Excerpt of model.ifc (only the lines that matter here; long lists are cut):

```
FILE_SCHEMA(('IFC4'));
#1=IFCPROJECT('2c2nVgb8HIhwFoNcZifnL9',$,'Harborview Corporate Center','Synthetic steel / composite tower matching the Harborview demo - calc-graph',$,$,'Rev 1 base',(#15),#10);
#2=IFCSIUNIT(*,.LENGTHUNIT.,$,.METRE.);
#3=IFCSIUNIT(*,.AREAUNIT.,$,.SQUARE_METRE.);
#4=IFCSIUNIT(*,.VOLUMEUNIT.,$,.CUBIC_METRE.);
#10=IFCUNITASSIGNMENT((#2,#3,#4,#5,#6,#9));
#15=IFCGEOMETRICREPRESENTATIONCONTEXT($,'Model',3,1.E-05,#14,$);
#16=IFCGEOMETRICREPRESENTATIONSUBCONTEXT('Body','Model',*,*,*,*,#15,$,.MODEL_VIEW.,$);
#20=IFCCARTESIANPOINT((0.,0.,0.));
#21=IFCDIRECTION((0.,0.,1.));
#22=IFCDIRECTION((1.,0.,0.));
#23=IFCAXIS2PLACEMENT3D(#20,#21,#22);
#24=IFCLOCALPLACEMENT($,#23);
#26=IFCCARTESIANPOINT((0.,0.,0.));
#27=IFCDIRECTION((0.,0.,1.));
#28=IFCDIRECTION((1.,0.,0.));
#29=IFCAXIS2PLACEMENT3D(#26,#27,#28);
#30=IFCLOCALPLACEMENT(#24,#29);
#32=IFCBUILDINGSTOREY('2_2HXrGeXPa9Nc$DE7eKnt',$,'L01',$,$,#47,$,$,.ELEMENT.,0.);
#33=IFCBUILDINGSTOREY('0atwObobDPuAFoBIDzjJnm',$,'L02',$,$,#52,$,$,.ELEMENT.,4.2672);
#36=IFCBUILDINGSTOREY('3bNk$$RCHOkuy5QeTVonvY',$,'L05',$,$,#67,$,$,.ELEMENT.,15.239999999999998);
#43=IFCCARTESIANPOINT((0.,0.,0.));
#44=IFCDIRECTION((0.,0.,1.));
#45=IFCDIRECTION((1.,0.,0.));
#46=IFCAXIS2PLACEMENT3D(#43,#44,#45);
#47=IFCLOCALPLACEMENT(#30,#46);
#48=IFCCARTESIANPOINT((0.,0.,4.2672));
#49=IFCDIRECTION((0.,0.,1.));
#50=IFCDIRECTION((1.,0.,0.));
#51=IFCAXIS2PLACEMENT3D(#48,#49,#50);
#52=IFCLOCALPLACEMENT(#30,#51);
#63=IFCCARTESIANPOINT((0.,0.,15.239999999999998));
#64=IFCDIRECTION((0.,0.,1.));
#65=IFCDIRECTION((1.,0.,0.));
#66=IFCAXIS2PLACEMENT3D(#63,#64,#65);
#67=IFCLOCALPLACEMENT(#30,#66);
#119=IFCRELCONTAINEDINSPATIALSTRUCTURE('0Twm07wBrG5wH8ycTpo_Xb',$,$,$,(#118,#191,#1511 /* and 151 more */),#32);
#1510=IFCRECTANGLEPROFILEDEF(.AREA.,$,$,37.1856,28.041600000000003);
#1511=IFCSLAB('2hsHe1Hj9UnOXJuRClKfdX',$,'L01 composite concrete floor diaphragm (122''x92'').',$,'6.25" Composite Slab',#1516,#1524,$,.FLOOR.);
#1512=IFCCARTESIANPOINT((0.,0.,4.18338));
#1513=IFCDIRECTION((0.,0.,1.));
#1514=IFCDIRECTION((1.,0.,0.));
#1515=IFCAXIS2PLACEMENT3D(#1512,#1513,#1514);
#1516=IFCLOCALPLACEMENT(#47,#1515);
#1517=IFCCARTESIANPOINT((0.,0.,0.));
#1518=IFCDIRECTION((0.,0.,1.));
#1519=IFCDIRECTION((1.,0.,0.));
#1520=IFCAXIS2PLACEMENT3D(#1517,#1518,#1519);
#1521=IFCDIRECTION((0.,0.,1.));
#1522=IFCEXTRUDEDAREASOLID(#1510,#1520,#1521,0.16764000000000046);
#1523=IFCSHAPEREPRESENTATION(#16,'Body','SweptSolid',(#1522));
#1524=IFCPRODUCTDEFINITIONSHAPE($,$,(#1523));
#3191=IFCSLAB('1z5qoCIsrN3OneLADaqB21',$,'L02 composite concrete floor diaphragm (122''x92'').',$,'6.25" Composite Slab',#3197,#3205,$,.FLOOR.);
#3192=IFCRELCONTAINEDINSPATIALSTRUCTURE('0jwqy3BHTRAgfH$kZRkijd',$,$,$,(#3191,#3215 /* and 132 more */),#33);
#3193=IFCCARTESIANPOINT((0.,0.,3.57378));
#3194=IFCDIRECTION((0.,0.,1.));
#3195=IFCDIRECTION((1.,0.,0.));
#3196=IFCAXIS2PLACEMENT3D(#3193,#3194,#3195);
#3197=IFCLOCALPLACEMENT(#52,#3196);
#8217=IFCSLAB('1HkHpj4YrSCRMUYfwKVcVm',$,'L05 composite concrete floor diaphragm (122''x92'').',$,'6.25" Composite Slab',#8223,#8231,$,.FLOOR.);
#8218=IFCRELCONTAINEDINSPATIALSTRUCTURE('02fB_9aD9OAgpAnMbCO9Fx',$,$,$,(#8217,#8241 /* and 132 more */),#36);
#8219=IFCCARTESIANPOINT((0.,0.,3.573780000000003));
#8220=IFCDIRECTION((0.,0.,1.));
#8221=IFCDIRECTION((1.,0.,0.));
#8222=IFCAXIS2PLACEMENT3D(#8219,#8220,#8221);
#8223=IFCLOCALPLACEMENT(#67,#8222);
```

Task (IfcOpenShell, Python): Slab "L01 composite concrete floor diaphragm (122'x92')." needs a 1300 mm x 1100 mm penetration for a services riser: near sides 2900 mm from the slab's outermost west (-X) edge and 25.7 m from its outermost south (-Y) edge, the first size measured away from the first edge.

```python
import numpy as np
import ifcopenshell
import ifcopenshell.api.feature
import ifcopenshell.api.geometry
import ifcopenshell.api.root
import ifcopenshell.geom
import ifcopenshell.util.placement
import ifcopenshell.util.representation
import ifcopenshell.util.shape
import ifcopenshell.util.unit

model = ifcopenshell.open("model.ifc")
unit_scale = ifcopenshell.util.unit.calculate_unit_scale(model)
settings = ifcopenshell.geom.settings()


def volume(element):
    """Net volume in cubic metres, openings subtracted."""
    shape = ifcopenshell.geom.create_shape(settings, element)
    return ifcopenshell.util.shape.get_volume(shape.geometry)


slab = model.by_guid("2hsHe1Hj9UnOXJuRClKfdX")
before = volume(slab)

# Extent in the slab's own axes, in metres. The edges named are its -X and -Y sides.
slab_shape = ifcopenshell.geom.create_shape(settings, slab)
vertices = ifcopenshell.util.shape.get_vertices(slab_shape.geometry)
x_min, y_min, bottom = vertices.min(axis=0)
top = vertices[:, 2].max()

opening = ifcopenshell.api.root.create_entity(model, ifc_class="IfcOpeningElement", name="Services riser opening", predefined_type="OPENING")
context = ifcopenshell.util.representation.get_context(model, "Model", "Body", "MODEL_VIEW")
width, depth = 1.3, 1.1
outline = [(0.0, 0.0), (width, 0.0), (width, depth), (0.0, depth), (0.0, 0.0)]
# Overshoot both faces by 50 mm so the cut is clean.
shape = ifcopenshell.api.geometry.add_slab_representation(
    model, context=context, depth=top - bottom + 0.1, polyline=outline
)
ifcopenshell.api.geometry.assign_representation(model, product=opening, representation=shape)

matrix = ifcopenshell.util.placement.get_local_placement(slab.ObjectPlacement)
matrix[:, 3] = matrix @ np.append(np.array([x_min + 2.9, y_min + 25.7, bottom - 0.05]) / unit_scale, 1.0)
ifcopenshell.api.geometry.edit_object_placement(model, product=opening, matrix=matrix, is_si=False)
ifcopenshell.api.feature.add_feature(model, feature=opening, element=slab)

after = volume(slab)

print(f"slab volume {before:.3f} -> {after:.3f} m3")

model.write("model_v2.ifc")
```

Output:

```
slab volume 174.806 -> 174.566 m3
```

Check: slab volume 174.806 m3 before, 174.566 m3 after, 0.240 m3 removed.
